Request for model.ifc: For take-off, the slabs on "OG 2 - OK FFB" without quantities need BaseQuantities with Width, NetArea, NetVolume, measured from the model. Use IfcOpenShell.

First a look at what the model holds.

```python
import ifcopenshell
import ifcopenshell.util.element
import ifcopenshell.util.unit

model = ifcopenshell.open("model.ifc")
print(model.schema)
for unit_type in ("LENGTHUNIT", "AREAUNIT", "VOLUMEUNIT"):
    print(unit_type, ifcopenshell.util.unit.calculate_unit_scale(model, unit_type))
storey = next(s for s in model.by_type("IfcBuildingStorey") if s.Name == "OG 2 - OK FFB")
slabs = [e for e in ifcopenshell.util.element.get_decomposition(storey) if e.is_a("IfcSlab")]
for e in sorted(slabs, key=lambda e: e.id()):
    print(e.id(), e.is_a(), e.Name, list(ifcopenshell.util.element.get_psets(e, qtos_only=True)), sep=" | ")
```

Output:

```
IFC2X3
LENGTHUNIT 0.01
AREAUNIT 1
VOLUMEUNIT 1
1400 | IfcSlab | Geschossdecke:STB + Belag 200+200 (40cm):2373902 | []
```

```python
import ifcopenshell
import ifcopenshell.api.pset
import ifcopenshell.geom
import ifcopenshell.util.element
import ifcopenshell.util.shape
import ifcopenshell.util.unit

model = ifcopenshell.open("model.ifc")
unit_scale = ifcopenshell.util.unit.calculate_unit_scale(model)
area_scale = ifcopenshell.util.unit.calculate_unit_scale(model, "AREAUNIT")
volume_scale = ifcopenshell.util.unit.calculate_unit_scale(model, "VOLUMEUNIT")
settings = ifcopenshell.geom.settings()

storey = next(s for s in model.by_type("IfcBuildingStorey") if s.Name == "OG 2 - OK FFB")
slabs = [e for e in ifcopenshell.util.element.get_decomposition(storey) if e.is_a("IfcSlab")]

for e in sorted(slabs, key=lambda e: e.id()):
    if ifcopenshell.util.element.get_psets(e, qtos_only=True, should_inherit=False):
        continue
    # Geometry comes back in metres, in the element's own axes.
    shape = ifcopenshell.geom.create_shape(settings, e)
    values = {
        "Width": ifcopenshell.util.shape.get_z(shape.geometry) / unit_scale,
        "NetArea": ifcopenshell.util.shape.get_footprint_area(shape.geometry) / area_scale,
        "NetVolume": ifcopenshell.util.shape.get_volume(shape.geometry) / volume_scale,
    }
    qto = ifcopenshell.api.pset.add_qto(model, product=e, name="BaseQuantities")
    ifcopenshell.api.pset.edit_qto(model, qto=qto, properties=values)
    print(e.id(), {k: round(v, 3) for k, v in values.items()})

model.write("model-out.ifc")
```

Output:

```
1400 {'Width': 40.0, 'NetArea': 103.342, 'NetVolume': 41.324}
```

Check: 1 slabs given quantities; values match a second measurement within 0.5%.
